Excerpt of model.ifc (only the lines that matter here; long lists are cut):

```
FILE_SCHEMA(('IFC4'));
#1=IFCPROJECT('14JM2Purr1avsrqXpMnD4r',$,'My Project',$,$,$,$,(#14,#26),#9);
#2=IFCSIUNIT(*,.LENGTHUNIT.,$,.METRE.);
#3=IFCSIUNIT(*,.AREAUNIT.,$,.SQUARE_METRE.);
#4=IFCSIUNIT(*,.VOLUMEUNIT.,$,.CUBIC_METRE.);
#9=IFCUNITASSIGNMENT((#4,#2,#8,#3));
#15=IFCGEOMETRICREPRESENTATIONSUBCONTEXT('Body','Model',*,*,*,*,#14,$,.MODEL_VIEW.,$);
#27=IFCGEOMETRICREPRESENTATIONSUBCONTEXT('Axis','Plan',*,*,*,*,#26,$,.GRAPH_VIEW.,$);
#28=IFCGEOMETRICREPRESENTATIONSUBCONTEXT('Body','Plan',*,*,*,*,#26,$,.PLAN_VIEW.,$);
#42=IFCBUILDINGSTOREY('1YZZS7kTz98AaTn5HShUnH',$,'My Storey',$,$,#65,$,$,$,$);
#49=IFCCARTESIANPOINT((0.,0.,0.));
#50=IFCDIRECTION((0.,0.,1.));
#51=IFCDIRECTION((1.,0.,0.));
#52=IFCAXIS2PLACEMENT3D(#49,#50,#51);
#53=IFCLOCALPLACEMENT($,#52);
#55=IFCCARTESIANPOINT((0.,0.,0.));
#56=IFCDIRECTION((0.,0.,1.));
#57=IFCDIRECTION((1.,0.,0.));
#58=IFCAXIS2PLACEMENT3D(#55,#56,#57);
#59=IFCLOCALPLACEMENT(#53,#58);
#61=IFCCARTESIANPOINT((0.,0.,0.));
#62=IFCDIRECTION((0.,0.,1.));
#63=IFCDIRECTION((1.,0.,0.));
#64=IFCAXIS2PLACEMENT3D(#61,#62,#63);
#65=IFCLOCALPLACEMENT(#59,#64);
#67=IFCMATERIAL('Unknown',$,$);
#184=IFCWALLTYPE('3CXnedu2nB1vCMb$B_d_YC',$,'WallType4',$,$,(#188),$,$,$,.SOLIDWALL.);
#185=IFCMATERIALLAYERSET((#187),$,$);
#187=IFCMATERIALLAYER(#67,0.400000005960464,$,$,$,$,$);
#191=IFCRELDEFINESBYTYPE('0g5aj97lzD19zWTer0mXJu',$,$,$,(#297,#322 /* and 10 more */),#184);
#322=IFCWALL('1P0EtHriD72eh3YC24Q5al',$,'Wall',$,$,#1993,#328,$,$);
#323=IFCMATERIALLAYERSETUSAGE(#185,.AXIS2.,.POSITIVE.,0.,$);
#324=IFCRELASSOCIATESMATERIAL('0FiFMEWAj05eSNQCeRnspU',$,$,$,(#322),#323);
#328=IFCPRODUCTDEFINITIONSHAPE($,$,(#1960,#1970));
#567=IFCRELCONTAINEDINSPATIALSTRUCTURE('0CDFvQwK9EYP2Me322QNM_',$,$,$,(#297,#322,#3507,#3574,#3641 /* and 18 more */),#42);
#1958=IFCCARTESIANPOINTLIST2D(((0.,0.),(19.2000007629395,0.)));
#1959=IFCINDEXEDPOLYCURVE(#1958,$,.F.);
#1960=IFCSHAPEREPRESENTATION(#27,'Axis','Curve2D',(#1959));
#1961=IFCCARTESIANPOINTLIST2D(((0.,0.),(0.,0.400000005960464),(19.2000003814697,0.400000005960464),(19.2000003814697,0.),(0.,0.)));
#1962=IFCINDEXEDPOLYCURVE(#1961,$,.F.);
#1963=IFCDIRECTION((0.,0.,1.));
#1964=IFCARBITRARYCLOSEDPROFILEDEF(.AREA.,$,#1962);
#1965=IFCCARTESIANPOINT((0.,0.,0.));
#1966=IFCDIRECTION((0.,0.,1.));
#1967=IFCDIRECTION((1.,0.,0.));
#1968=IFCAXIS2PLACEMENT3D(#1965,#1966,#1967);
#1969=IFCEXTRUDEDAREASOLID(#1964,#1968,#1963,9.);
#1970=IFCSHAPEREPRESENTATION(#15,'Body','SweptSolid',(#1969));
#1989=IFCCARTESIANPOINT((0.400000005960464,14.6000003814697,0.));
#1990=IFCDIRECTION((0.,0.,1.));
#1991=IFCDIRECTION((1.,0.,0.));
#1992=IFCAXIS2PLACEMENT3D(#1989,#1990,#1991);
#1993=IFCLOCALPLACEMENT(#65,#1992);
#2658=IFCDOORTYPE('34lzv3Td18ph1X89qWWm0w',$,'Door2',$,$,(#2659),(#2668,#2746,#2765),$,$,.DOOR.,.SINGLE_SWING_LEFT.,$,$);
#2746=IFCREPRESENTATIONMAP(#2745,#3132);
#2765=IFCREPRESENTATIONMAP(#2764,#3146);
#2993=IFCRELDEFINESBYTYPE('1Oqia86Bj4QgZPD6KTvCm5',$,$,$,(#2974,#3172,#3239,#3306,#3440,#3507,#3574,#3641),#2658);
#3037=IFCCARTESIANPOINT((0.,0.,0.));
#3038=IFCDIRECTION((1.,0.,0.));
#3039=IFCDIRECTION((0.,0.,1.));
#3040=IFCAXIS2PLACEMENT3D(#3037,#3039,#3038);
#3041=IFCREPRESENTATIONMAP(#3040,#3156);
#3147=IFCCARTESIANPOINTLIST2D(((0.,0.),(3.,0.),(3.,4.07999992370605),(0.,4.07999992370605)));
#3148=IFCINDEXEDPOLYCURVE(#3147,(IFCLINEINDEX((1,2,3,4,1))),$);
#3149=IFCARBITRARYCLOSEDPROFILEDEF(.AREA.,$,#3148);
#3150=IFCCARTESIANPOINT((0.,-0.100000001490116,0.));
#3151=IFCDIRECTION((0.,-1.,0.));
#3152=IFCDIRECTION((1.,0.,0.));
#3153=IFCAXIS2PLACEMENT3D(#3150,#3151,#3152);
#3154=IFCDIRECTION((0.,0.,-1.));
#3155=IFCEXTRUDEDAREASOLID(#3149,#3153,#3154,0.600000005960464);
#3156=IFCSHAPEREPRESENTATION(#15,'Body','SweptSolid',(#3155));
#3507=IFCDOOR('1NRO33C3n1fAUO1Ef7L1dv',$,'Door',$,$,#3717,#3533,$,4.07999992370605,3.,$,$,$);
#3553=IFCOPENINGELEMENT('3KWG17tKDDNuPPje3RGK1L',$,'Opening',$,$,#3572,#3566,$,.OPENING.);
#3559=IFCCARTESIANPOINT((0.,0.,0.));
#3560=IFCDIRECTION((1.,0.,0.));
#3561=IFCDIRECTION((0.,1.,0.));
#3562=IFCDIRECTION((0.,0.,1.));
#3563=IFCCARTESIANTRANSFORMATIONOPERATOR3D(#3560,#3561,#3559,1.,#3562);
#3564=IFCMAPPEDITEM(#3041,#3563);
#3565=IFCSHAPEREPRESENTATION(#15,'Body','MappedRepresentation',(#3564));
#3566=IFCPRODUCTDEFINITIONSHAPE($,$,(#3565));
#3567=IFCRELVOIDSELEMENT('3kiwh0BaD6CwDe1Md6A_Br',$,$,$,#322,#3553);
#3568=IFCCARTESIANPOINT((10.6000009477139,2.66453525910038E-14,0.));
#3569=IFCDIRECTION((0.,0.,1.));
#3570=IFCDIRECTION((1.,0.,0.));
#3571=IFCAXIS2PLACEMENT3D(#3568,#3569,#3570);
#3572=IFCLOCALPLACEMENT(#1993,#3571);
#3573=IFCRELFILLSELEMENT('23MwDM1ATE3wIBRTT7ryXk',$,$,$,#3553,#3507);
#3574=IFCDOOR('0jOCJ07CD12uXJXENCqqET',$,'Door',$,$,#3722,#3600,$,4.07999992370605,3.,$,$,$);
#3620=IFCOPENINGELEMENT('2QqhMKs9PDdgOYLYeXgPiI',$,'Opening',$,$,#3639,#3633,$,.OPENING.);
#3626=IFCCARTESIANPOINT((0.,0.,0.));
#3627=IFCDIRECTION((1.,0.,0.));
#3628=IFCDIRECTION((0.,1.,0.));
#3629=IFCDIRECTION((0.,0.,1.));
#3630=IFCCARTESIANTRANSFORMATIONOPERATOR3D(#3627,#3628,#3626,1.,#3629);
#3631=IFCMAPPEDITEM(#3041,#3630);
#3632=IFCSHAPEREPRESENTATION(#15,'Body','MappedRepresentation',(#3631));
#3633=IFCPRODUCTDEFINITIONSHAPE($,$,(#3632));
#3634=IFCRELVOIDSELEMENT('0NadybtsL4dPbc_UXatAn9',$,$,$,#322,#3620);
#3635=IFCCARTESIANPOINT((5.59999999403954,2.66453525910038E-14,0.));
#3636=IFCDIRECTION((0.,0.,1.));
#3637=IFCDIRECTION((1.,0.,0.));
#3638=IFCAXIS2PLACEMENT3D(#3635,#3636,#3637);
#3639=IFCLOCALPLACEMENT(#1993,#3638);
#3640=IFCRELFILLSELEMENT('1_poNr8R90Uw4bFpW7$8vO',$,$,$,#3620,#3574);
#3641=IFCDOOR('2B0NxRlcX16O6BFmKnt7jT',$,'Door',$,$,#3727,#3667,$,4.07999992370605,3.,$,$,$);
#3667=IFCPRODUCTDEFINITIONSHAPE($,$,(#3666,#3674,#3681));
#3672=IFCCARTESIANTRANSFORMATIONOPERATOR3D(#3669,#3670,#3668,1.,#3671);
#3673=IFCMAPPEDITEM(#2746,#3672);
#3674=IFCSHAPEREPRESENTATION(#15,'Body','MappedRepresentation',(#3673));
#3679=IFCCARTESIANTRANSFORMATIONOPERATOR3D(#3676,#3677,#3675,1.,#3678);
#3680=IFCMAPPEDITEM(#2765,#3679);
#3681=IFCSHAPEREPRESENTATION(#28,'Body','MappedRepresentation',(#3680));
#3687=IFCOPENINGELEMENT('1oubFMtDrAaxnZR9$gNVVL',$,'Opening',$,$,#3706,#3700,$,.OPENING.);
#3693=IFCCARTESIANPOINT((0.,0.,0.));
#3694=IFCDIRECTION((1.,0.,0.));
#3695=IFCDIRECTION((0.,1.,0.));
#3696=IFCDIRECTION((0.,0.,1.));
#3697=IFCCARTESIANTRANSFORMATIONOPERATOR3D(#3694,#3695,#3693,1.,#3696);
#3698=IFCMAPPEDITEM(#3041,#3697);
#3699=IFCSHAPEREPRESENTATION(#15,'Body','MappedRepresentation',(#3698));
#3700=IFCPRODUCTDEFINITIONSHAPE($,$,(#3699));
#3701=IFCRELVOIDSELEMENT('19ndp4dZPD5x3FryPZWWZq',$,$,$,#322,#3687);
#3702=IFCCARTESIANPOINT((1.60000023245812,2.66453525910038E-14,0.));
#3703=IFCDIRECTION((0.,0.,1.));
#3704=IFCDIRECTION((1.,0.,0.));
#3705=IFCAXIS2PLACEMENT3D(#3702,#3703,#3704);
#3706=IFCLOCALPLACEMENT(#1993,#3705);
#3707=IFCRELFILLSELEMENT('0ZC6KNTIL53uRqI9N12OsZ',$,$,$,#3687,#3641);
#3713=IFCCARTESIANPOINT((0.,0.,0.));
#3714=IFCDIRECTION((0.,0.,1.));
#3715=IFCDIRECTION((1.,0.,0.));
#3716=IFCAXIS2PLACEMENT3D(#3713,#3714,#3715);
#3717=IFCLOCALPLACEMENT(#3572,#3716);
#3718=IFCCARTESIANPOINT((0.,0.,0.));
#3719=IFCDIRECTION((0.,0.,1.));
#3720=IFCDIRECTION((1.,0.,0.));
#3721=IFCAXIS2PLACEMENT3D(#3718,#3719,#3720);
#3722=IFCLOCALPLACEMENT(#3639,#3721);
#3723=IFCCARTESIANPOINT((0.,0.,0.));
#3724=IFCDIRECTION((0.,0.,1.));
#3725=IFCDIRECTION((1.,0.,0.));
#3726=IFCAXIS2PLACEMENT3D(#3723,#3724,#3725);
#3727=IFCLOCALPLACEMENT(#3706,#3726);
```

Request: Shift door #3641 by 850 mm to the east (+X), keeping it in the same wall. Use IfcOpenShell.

```python
import ifcopenshell
import ifcopenshell.api.geometry
import ifcopenshell.util.placement

model = ifcopenshell.open("model.ifc")

door = model.by_guid("2B0NxRlcX16O6BFmKnt7jT")
opening = door.FillsVoids[0].RelatingOpeningElement
wall = opening.VoidsElements[0].RelatingBuildingElement

wall_matrix = ifcopenshell.util.placement.get_local_placement(wall.ObjectPlacement)
shift = wall_matrix[:3, 0] * 0.85
before = ifcopenshell.util.placement.get_local_placement(door.ObjectPlacement)[:3, 3].copy()

# The door is placed relative to its opening, so it follows when the opening moves.
matrix = ifcopenshell.util.placement.get_local_placement(opening.ObjectPlacement)
matrix[:3, 3] += shift
ifcopenshell.api.geometry.edit_object_placement(
    model, product=opening, matrix=matrix, is_si=False, should_transform_children=True
)

after = ifcopenshell.util.placement.get_local_placement(door.ObjectPlacement)[:3, 3]
print("door moved by", (after - before).round(3) + 0.0)

model.write("model_edited.ifc")
```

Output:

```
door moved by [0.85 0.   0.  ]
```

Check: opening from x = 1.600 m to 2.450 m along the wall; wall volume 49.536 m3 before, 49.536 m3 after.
